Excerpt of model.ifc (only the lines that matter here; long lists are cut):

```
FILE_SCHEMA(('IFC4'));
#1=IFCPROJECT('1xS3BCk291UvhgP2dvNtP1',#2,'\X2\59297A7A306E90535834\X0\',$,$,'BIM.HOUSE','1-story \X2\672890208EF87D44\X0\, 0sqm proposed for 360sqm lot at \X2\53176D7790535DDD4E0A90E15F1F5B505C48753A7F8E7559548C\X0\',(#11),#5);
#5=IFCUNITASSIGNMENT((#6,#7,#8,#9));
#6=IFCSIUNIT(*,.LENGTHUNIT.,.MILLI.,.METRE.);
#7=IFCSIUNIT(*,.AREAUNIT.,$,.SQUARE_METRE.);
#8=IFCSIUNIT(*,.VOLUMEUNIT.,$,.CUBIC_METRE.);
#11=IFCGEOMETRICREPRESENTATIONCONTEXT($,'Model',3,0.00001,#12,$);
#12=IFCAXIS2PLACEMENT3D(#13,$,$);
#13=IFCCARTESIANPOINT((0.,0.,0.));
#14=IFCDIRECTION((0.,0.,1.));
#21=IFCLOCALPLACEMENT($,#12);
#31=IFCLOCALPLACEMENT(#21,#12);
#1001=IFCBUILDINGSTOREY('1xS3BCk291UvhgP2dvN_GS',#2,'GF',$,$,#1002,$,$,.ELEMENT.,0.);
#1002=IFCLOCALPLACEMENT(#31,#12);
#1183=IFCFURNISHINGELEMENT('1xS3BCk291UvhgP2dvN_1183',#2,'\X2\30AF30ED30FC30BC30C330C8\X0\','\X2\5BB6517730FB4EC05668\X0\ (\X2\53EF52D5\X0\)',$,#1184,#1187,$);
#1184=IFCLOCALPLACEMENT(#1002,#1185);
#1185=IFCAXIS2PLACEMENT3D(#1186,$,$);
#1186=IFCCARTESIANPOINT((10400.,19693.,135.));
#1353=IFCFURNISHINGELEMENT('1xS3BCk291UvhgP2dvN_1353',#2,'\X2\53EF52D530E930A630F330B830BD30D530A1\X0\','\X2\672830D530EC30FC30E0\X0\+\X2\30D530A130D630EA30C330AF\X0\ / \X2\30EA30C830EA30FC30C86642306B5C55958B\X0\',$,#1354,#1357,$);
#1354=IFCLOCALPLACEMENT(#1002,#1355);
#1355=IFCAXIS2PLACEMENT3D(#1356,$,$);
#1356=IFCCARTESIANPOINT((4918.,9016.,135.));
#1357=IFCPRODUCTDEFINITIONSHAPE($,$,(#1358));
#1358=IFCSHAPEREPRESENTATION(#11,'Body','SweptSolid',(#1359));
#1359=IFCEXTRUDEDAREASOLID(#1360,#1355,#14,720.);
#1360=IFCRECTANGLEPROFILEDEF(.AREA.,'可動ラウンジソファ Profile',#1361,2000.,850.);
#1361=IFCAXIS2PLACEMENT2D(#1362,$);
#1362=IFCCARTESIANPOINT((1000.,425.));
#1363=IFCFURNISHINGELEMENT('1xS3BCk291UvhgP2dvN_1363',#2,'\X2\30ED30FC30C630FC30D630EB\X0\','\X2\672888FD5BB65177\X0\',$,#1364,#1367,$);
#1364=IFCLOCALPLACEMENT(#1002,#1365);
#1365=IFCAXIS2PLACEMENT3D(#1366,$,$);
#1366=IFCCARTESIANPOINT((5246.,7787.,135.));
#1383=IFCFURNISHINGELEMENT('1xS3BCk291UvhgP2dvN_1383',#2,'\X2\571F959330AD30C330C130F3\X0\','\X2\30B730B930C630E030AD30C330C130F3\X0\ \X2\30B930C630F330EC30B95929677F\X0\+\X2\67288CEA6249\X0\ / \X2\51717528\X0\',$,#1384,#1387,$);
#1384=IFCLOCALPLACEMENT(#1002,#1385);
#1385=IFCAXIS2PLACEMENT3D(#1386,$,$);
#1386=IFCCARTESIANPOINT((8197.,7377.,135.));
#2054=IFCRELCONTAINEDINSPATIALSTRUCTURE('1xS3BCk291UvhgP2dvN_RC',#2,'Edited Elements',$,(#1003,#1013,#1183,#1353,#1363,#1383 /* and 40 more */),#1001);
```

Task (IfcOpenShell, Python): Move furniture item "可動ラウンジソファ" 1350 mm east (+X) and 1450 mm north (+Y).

```python
import ifcopenshell
import ifcopenshell.api.geometry
import ifcopenshell.util.placement
import ifcopenshell.util.unit

model = ifcopenshell.open("model.ifc")
unit_scale = ifcopenshell.util.unit.calculate_unit_scale(model)

item = model.by_guid("1xS3BCk291UvhgP2dvN_1353")
matrix = ifcopenshell.util.placement.get_local_placement(item.ObjectPlacement)
matrix[0, 3] += 1.35 / unit_scale
matrix[1, 3] += 1.45 / unit_scale
ifcopenshell.api.geometry.edit_object_placement(model, product=item, matrix=matrix, is_si=False)

print(ifcopenshell.util.placement.get_local_placement(item.ObjectPlacement).round(3) + 0.0)

model.write("model_edited.ifc")
```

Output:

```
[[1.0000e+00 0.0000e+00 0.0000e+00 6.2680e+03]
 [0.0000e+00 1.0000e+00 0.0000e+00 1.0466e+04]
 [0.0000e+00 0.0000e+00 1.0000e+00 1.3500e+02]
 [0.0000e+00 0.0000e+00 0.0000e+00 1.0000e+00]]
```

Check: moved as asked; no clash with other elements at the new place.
